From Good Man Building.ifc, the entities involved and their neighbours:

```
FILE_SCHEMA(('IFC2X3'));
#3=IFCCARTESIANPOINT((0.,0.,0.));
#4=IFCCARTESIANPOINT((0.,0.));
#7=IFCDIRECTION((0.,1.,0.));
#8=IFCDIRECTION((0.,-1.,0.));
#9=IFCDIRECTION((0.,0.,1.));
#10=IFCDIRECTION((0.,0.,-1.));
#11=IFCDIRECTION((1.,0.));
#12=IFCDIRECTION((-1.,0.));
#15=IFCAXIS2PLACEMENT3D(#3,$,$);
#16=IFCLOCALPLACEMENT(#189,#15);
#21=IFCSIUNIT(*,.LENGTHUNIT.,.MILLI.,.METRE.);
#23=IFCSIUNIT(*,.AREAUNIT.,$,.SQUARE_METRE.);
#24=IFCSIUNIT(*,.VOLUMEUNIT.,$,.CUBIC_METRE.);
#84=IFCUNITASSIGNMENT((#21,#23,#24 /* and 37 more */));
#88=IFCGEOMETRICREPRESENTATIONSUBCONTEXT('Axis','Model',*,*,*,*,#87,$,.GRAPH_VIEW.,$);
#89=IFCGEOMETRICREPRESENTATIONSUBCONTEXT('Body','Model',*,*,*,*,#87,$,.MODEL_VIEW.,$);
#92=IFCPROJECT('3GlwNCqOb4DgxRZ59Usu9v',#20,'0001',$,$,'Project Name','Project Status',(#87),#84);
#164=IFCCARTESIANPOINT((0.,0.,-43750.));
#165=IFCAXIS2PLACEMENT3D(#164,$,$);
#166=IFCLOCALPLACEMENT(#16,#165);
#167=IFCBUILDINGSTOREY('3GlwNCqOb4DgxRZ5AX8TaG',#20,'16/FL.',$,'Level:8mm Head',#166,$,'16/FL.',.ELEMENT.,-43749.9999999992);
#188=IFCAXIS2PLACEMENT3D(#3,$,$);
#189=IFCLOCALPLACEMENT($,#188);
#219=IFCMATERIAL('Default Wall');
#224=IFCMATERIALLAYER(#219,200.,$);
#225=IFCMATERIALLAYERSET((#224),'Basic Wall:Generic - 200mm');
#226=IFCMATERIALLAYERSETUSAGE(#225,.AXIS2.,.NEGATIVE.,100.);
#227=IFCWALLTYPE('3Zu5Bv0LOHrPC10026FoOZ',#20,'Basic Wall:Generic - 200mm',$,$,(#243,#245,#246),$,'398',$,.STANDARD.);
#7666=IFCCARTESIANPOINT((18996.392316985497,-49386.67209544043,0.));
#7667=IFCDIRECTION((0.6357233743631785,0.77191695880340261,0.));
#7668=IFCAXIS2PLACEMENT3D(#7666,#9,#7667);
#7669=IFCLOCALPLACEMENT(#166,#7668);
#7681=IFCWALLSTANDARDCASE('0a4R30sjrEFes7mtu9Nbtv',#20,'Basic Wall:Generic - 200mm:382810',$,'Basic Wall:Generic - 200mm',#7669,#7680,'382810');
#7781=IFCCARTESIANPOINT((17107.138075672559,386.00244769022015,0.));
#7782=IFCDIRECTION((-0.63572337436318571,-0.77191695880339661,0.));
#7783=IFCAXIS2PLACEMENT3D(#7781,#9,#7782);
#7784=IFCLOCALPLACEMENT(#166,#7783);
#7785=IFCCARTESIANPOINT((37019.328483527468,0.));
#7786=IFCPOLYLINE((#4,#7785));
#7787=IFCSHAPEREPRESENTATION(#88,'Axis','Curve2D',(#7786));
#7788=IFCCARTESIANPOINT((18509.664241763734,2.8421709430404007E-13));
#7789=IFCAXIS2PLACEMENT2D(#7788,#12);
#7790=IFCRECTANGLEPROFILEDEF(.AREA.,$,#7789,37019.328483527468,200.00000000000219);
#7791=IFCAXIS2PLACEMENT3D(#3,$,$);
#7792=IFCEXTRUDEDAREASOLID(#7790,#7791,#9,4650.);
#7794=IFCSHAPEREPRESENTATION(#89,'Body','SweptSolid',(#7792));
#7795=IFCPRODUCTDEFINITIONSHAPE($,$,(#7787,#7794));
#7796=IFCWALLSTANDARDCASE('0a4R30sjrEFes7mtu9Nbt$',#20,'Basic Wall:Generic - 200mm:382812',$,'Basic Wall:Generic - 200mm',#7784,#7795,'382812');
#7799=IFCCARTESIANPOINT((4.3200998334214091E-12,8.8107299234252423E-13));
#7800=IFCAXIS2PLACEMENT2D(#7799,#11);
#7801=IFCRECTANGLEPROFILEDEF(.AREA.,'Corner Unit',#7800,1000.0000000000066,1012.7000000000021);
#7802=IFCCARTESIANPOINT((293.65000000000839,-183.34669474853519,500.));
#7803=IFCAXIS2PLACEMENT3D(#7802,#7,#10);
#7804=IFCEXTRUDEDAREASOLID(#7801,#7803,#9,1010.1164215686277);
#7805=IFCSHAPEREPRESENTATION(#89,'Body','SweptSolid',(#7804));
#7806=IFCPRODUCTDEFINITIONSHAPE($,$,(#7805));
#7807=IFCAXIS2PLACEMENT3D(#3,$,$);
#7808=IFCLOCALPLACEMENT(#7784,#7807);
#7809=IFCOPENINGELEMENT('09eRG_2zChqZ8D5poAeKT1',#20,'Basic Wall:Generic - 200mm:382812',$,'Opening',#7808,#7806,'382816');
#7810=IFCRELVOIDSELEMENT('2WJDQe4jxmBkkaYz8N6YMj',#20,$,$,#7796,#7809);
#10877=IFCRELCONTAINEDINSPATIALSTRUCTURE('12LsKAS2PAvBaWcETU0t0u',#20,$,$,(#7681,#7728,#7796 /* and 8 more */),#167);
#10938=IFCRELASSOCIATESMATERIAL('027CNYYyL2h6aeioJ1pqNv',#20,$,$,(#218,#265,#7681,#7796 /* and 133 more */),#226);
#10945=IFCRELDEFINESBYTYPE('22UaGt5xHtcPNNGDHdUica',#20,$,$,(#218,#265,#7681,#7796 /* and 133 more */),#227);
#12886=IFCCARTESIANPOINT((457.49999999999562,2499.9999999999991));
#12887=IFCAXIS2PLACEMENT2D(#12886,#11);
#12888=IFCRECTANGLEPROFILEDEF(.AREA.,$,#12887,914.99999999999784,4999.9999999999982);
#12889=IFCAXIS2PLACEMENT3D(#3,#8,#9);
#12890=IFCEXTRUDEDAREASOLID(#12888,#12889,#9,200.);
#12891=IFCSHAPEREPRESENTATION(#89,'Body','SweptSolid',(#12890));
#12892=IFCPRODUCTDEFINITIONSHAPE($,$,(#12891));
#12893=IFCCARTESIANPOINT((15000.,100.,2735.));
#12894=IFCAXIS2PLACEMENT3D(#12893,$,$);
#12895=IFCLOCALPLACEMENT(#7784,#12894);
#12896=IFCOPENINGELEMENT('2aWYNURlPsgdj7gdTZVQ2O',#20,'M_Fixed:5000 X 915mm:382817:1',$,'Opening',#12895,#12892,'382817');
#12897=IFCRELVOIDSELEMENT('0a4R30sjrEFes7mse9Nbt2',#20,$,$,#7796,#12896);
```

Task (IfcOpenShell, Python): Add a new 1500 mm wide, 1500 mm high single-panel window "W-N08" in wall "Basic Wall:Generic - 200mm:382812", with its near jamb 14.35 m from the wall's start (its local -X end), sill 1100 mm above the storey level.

```python
import numpy as np
import ifcopenshell
import ifcopenshell.api.feature
import ifcopenshell.api.geometry
import ifcopenshell.api.root
import ifcopenshell.api.spatial
import ifcopenshell.api.type
import ifcopenshell.geom
import ifcopenshell.util.element
import ifcopenshell.util.placement
import ifcopenshell.util.representation
import ifcopenshell.util.shape
import ifcopenshell.util.unit

model = ifcopenshell.open("Good Man Building.ifc")
unit_scale = ifcopenshell.util.unit.calculate_unit_scale(model)
settings = ifcopenshell.geom.settings()


def volume(element):
    """Net volume in cubic metres, openings subtracted."""
    shape = ifcopenshell.geom.create_shape(settings, element)
    return ifcopenshell.util.shape.get_volume(shape.geometry)


wall = model.by_id(7796)
storey = ifcopenshell.util.element.get_container(wall, ifc_class="IfcBuildingStorey")
context = ifcopenshell.util.representation.get_context(model, "Model", "Body", "MODEL_VIEW")
before = volume(wall)

width, height, from_end, sill = 1.5, 1.5, 14.35, 1.1  # metres

# The wall runs along its own X axis, and the end named is its -X end.
wall_shape = ifcopenshell.geom.create_shape(settings, wall)
x, y, z = ifcopenshell.util.shape.get_vertices(wall_shape.geometry).T
start = x.min() + from_end
face, thickness = float(y.min()), float(y.max() - y.min())
wall_matrix = ifcopenshell.util.placement.get_local_placement(wall.ObjectPlacement)
level = ifcopenshell.util.placement.get_local_placement(storey.ObjectPlacement)[2, 3]


def in_wall(x, y):
    """Placement at x, y metres in the wall's axes, at sill height."""
    matrix = wall_matrix.copy()
    matrix[:, 3] = wall_matrix @ np.array([x / unit_scale, y / unit_scale, 0.0, 1.0])
    matrix[2, 3] = level + sill / unit_scale
    return matrix


# Opening: a box that overshoots both wall faces by 50 mm.
opening = ifcopenshell.api.root.create_entity(model, ifc_class="IfcOpeningElement")
box = ifcopenshell.api.geometry.add_wall_representation(
    model, context=context, length=width, height=height, thickness=thickness + 0.1
)
ifcopenshell.api.geometry.assign_representation(model, product=opening, representation=box)
ifcopenshell.api.geometry.edit_object_placement(model, product=opening, matrix=in_wall(start, face - 0.05), is_si=False)
ifcopenshell.api.feature.add_feature(model, feature=opening, element=wall)

window = ifcopenshell.api.root.create_entity(model, ifc_class="IfcWindow", name="W-N08")
window.OverallWidth, window.OverallHeight = width / unit_scale, height / unit_scale
body = ifcopenshell.api.geometry.add_window_representation(
    model,
    context=context,
    overall_width=window.OverallWidth,
    overall_height=window.OverallHeight,
    partition_type="SINGLE_PANEL",
)
ifcopenshell.api.geometry.assign_representation(model, product=window, representation=body)
ifcopenshell.api.spatial.assign_container(model, products=[window], relating_structure=storey)
fills = ifcopenshell.api.feature.add_filling(model, opening=opening, element=window)
fills.OwnerHistory = window.OwnerHistory  # required in IFC2X3

# IFC2X3 keeps the operation on the window style.
style = ifcopenshell.api.root.create_entity(model, ifc_class="IfcWindowStyle", name="W-N08")
style.OperationType, style.ConstructionType = "SINGLE_PANEL", "NOTDEFINED"
style.ParameterTakesPrecedence = style.Sizeable = False
ifcopenshell.api.type.assign_type(model, related_objects=[window], relating_type=style)

# Centre the window in the wall's thickness.
ifcopenshell.api.geometry.edit_object_placement(model, product=window, matrix=in_wall(start, face), is_si=False)
window_shape = ifcopenshell.geom.create_shape(settings, window)
depth = ifcopenshell.util.shape.get_vertices(window_shape.geometry)[:, 1]
offset = face + thickness / 2 - (depth.min() + depth.max()) / 2
ifcopenshell.api.geometry.edit_object_placement(model, product=window, matrix=in_wall(start, offset), is_si=False)

after = volume(wall)

print(f"wall volume {before:.3f} -> {after:.3f} m3")

model.write("Good Man Building-out.ifc")
```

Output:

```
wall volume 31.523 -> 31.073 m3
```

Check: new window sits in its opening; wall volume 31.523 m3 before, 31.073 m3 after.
